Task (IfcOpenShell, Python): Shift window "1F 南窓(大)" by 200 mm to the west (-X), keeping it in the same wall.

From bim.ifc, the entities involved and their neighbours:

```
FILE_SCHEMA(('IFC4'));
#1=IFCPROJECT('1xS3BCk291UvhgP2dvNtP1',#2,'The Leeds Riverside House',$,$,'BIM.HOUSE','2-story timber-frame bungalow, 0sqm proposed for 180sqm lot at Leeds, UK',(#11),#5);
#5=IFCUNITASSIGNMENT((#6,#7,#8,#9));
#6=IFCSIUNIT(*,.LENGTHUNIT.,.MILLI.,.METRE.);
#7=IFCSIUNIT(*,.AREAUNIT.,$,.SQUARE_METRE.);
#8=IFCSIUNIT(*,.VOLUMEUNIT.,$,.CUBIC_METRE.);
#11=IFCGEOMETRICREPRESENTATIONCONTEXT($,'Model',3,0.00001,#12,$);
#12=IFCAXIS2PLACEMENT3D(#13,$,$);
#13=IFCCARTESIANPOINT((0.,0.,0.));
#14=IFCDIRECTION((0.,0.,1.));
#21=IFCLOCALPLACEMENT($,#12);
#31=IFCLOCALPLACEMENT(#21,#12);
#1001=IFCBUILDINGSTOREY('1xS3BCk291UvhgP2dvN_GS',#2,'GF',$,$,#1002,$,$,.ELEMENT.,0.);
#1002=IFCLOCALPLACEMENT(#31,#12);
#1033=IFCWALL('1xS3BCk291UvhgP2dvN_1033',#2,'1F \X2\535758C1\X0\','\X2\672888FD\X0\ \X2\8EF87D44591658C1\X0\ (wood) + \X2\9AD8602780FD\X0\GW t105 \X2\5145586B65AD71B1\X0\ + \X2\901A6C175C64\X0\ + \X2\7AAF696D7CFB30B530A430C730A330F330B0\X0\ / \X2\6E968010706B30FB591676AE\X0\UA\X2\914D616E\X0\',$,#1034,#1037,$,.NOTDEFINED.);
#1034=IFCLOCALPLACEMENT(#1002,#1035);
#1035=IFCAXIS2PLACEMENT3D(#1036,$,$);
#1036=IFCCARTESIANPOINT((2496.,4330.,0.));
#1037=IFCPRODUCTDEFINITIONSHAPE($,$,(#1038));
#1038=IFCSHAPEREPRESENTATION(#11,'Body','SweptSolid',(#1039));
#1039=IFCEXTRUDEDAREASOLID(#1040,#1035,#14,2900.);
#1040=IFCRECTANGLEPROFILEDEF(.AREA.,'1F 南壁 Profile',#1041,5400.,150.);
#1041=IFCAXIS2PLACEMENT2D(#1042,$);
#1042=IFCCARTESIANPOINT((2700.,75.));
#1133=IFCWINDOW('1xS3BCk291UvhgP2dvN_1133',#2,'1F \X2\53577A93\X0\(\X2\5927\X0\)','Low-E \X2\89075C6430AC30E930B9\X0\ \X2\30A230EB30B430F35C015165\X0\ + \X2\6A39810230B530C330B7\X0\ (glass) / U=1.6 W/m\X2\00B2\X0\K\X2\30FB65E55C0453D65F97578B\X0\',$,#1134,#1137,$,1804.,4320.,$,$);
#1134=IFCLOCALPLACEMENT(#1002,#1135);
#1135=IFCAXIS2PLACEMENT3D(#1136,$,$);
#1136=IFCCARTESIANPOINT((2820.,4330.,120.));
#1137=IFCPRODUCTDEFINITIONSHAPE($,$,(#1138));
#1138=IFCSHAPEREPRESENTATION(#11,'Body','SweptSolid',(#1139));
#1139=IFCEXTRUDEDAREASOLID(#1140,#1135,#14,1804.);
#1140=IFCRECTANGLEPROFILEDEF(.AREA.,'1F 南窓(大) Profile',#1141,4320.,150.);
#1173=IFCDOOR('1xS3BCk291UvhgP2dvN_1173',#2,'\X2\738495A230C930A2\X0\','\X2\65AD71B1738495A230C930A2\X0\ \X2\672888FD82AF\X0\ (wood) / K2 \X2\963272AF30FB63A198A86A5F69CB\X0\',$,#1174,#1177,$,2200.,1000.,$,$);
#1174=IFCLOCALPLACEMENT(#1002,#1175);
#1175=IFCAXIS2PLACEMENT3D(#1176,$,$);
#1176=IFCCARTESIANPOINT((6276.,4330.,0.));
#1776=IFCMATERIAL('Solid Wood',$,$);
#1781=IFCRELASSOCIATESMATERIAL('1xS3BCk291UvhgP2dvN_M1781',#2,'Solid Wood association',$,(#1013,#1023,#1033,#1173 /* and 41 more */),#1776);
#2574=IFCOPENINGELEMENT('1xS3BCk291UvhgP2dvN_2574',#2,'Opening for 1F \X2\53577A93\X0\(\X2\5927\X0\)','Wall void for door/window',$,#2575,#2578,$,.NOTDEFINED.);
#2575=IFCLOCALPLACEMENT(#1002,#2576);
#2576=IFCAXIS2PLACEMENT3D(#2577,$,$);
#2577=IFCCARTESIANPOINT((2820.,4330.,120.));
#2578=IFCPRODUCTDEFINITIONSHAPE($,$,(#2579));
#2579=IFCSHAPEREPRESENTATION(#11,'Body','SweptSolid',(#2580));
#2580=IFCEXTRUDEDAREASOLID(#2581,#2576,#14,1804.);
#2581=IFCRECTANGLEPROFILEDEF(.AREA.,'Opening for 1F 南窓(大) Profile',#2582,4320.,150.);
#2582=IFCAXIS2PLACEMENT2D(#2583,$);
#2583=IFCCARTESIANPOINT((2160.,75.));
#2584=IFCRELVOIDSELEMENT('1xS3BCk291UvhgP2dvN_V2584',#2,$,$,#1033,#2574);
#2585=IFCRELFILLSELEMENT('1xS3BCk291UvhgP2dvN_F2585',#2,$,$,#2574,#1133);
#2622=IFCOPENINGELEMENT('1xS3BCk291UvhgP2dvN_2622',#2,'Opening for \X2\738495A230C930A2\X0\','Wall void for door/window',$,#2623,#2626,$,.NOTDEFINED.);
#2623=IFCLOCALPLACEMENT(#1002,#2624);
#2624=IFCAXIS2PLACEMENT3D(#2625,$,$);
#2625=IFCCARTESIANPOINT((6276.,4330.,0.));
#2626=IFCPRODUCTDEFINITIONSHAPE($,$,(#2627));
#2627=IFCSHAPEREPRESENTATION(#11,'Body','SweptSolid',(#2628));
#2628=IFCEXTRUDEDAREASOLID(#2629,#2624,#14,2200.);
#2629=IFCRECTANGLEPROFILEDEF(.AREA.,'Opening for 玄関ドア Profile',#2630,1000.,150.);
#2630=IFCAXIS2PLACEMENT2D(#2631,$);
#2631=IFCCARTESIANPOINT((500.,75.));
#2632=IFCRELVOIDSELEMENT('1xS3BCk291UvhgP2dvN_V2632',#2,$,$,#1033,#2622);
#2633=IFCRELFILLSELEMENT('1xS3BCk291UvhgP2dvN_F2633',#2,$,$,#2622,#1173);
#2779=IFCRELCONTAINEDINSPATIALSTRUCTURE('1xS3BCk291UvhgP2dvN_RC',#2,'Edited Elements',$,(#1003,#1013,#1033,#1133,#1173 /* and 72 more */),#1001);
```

```python
import ifcopenshell
import ifcopenshell.api.geometry
import ifcopenshell.util.placement

model = ifcopenshell.open("bim.ifc")

window = model.by_guid("1xS3BCk291UvhgP2dvN_1133")
opening = window.FillsVoids[0].RelatingOpeningElement
wall = opening.VoidsElements[0].RelatingBuildingElement

wall_matrix = ifcopenshell.util.placement.get_local_placement(wall.ObjectPlacement)
shift = wall_matrix[:3, 0] * -200.0
before = ifcopenshell.util.placement.get_local_placement(window.ObjectPlacement)[:3, 3].copy()

# The window is not placed relative to its opening, so move both.
for product in (opening, window):
    matrix = ifcopenshell.util.placement.get_local_placement(product.ObjectPlacement)
    matrix[:3, 3] += shift
    ifcopenshell.api.geometry.edit_object_placement(model, product=product, matrix=matrix, is_si=False)

after = ifcopenshell.util.placement.get_local_placement(window.ObjectPlacement)[:3, 3]
print("window moved by", (after - before).round(3) + 0.0)

model.write("bim_updated.ifc")
```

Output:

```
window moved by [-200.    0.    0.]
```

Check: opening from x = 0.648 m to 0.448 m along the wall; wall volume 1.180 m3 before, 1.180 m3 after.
